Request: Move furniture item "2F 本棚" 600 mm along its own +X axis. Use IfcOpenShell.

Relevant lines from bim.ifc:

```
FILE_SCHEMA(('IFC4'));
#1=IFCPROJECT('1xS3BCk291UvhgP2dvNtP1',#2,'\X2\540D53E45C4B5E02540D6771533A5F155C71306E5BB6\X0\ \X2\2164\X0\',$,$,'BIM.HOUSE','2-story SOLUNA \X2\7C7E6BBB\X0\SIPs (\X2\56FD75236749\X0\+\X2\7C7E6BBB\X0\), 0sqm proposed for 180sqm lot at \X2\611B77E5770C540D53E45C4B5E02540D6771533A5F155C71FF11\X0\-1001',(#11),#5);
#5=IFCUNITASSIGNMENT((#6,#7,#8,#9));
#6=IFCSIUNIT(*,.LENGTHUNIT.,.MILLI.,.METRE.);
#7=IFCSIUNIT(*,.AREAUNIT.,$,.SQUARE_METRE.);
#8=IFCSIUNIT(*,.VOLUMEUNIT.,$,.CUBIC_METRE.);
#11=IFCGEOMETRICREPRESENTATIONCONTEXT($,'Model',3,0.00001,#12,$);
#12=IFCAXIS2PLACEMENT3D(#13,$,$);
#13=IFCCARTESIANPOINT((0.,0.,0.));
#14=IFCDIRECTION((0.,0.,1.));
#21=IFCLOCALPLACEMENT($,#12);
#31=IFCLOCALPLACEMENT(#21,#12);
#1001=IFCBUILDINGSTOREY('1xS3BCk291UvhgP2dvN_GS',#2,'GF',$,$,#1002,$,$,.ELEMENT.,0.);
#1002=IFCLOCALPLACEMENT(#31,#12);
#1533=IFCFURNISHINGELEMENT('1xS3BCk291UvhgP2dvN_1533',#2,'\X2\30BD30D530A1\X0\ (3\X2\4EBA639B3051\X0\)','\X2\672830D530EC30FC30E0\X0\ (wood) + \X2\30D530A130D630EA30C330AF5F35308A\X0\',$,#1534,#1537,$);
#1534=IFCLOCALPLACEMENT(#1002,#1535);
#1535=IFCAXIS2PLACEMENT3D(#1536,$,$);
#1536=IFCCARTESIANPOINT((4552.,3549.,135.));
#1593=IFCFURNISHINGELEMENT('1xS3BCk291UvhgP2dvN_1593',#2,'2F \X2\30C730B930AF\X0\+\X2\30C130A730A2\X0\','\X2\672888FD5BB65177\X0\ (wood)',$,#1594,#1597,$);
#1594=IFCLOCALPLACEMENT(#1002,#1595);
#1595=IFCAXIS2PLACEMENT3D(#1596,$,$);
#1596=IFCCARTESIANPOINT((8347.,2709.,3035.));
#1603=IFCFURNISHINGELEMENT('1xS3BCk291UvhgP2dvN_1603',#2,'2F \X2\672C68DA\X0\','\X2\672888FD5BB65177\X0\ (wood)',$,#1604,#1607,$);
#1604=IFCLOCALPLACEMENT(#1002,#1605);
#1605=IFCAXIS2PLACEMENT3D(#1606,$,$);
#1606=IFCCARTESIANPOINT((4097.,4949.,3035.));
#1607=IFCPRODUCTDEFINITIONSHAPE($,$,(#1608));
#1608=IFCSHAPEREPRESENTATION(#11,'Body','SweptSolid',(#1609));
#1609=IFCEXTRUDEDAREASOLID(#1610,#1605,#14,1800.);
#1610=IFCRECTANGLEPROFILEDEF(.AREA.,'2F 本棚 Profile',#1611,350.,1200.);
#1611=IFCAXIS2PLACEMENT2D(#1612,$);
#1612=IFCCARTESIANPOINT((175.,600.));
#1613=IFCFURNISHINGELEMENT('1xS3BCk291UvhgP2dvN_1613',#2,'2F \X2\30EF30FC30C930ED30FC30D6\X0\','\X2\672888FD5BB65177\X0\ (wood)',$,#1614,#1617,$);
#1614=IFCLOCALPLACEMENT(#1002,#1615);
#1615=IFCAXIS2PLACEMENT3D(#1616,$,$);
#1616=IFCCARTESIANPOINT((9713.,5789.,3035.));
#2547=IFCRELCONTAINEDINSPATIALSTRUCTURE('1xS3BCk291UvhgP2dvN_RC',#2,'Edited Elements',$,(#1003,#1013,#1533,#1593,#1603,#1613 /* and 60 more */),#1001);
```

```python
import ifcopenshell
import ifcopenshell.api.geometry
import ifcopenshell.util.placement

model = ifcopenshell.open("bim.ifc")

item = model.by_guid("1xS3BCk291UvhgP2dvN_1603")
matrix = ifcopenshell.util.placement.get_local_placement(item.ObjectPlacement)
matrix[:3, 3] += matrix[:3, 0] * 600.0
ifcopenshell.api.geometry.edit_object_placement(model, product=item, matrix=matrix, is_si=False)

print(ifcopenshell.util.placement.get_local_placement(item.ObjectPlacement).round(3) + 0.0)

model.write("bim_v2.ifc")
```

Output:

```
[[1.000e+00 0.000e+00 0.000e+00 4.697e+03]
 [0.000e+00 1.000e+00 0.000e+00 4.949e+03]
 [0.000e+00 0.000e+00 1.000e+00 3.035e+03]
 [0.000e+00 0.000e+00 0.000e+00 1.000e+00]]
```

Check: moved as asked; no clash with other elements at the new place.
